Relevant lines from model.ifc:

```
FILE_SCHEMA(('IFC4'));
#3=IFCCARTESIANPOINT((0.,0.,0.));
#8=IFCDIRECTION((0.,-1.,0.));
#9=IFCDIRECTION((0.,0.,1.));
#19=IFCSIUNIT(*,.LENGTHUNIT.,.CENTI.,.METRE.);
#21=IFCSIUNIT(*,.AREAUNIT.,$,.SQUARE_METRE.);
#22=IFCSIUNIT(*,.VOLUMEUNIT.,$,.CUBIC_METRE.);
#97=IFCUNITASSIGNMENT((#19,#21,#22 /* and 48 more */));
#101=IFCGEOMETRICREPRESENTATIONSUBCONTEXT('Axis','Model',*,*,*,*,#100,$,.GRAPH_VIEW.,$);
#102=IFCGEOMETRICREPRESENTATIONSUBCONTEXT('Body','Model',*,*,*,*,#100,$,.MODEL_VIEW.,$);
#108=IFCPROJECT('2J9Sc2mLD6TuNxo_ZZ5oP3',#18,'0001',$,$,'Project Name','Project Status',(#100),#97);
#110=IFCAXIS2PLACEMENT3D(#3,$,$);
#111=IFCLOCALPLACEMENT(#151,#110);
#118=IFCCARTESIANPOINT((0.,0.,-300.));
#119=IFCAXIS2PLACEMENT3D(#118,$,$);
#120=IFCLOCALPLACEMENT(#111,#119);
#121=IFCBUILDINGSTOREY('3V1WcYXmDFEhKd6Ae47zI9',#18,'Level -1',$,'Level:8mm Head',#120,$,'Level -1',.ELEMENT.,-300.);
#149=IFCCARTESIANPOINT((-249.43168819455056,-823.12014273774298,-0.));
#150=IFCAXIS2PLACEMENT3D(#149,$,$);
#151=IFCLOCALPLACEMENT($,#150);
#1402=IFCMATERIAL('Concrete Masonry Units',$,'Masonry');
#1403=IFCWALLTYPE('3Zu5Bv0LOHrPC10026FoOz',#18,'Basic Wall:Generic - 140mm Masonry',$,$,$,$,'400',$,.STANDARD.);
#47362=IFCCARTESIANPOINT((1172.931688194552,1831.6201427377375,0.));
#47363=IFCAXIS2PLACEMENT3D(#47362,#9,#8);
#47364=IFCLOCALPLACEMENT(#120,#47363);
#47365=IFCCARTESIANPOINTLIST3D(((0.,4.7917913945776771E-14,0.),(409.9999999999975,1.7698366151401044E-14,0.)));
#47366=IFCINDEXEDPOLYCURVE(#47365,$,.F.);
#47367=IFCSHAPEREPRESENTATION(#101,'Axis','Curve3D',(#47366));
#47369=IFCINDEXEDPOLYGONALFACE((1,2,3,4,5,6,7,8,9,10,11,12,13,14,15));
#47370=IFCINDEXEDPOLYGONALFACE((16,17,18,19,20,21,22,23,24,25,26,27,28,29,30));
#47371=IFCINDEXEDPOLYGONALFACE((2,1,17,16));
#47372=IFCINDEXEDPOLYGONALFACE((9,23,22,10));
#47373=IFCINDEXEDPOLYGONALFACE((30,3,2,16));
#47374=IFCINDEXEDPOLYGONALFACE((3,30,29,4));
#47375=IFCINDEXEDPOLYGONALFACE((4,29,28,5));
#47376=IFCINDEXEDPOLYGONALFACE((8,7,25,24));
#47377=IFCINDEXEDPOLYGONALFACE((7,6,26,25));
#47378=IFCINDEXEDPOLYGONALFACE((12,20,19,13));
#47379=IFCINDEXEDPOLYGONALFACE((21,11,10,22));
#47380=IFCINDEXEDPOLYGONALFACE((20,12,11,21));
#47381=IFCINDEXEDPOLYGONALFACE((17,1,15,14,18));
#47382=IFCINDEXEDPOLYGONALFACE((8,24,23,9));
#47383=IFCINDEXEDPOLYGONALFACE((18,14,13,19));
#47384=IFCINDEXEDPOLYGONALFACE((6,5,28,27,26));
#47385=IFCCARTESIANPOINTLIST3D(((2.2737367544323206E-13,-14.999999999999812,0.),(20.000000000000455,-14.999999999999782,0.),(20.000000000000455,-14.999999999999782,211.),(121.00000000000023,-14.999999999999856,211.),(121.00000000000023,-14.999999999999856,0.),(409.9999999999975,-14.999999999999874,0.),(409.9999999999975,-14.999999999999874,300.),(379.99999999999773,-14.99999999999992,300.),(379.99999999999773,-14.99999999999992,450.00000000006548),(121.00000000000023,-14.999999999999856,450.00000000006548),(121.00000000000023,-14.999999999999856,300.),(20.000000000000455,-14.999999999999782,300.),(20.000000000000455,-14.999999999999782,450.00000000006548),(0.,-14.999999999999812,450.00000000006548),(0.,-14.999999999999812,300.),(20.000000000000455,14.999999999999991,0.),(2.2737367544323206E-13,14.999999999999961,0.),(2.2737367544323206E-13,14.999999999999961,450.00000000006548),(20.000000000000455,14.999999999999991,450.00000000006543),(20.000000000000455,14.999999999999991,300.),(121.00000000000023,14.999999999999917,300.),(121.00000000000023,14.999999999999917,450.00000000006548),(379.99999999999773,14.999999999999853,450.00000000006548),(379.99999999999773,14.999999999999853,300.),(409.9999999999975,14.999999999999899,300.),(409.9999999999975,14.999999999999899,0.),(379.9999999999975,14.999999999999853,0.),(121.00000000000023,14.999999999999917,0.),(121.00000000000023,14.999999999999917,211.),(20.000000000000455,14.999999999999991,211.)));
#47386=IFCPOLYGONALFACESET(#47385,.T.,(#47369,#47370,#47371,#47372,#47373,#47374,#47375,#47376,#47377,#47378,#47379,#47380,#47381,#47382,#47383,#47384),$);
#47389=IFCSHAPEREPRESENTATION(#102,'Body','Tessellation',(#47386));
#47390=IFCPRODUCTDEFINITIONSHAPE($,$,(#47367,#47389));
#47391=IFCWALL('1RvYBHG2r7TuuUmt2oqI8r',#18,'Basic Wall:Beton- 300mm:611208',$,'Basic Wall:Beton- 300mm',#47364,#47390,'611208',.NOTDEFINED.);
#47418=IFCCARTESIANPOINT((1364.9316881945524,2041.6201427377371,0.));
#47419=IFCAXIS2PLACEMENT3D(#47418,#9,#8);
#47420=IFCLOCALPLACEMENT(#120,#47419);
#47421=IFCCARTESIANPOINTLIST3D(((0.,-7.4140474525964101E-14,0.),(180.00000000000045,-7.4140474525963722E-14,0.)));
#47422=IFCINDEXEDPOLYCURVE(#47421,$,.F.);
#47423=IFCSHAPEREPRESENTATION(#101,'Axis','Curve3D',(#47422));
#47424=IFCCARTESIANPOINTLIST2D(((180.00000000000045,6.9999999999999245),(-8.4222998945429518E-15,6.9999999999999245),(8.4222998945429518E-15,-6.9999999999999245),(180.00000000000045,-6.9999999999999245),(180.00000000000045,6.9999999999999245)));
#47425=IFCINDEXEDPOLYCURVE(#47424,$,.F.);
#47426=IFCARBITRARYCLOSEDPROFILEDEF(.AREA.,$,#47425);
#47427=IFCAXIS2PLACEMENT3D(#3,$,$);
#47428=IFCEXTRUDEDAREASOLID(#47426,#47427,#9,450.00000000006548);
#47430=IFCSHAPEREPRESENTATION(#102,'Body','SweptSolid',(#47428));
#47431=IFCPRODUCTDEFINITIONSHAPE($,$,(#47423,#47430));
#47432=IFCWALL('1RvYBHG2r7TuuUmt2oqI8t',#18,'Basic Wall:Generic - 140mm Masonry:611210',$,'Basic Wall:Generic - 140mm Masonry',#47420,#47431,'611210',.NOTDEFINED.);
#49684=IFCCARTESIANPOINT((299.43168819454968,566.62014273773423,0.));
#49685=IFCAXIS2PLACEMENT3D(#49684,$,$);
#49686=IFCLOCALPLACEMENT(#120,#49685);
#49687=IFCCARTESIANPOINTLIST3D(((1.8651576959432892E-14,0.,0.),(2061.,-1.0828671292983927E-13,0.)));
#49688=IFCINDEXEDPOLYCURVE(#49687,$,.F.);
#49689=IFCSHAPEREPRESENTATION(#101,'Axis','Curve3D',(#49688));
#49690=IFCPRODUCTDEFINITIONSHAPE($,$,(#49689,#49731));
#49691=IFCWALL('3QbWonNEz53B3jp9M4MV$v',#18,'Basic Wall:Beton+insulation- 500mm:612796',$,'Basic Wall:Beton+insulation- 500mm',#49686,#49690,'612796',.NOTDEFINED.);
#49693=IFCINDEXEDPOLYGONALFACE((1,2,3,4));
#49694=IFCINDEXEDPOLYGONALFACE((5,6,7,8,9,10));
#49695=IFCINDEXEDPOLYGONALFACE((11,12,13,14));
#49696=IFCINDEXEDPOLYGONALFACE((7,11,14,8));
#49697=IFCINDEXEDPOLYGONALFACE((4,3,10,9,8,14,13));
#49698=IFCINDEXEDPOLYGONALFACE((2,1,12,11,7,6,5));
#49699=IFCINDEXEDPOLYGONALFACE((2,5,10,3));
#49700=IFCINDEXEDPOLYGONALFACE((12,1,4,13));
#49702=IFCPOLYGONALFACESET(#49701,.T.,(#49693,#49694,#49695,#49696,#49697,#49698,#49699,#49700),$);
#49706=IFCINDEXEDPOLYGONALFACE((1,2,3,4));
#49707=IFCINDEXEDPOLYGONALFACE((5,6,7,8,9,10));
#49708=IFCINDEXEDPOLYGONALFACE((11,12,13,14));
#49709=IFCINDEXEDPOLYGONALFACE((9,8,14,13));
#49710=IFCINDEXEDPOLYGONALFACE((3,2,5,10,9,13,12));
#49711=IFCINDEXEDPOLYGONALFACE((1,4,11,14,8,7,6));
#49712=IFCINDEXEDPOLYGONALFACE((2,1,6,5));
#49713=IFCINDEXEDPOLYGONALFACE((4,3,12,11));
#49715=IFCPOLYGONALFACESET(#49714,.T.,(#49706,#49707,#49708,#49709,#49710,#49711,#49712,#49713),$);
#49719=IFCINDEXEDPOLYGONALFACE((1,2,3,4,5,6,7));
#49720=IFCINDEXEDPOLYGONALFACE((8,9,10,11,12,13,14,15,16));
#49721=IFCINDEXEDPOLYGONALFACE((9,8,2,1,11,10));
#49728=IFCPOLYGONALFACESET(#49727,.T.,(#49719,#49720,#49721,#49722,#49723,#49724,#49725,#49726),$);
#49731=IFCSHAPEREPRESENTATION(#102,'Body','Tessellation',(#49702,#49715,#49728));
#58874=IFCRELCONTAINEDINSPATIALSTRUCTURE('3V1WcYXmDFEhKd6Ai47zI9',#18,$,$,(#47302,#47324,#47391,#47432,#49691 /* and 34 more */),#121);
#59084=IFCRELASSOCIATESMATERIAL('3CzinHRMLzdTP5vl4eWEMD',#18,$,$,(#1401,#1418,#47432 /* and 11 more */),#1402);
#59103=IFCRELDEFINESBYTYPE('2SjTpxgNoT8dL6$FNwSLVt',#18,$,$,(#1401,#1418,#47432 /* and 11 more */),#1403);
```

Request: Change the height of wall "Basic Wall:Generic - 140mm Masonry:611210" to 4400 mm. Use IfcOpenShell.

```python
import ifcopenshell
import ifcopenshell.geom
import ifcopenshell.util.representation
import ifcopenshell.util.shape
import ifcopenshell.util.unit

model = ifcopenshell.open("model.ifc")
unit_scale = ifcopenshell.util.unit.calculate_unit_scale(model)
settings = ifcopenshell.geom.settings()


def volume(element):
    """Net volume in cubic metres, openings subtracted."""
    shape = ifcopenshell.geom.create_shape(settings, element)
    return ifcopenshell.util.shape.get_volume(shape.geometry)


wall = model.by_id(47432)
before = volume(wall)

body = ifcopenshell.util.representation.get_representation(wall, "Model", "Body")
solid = body.Items[0]
old_height = solid.Depth
solid.Depth = 4.4 / unit_scale
after = volume(wall)

print(f"height {old_height:g} -> {solid.Depth:g}, volume {before:.3f} -> {after:.3f} m3")

model.write("model-out.ifc")
```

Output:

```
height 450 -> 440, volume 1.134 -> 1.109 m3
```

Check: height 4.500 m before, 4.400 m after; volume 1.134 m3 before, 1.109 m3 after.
